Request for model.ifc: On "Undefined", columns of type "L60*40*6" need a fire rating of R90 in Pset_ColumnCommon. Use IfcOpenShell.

First a look at what the model holds.

```python
import ifcopenshell
import ifcopenshell.util.element

model = ifcopenshell.open("model.ifc")
print(model.schema)
storey = next(s for s in model.by_type("IfcBuildingStorey") if s.Name == "Undefined")
columns = [e for e in ifcopenshell.util.element.get_decomposition(storey) if e.is_a("IfcColumn")]
seen = {}
for e in columns:
    element_type = ifcopenshell.util.element.get_type(e)
    key = (element_type.Name if element_type != e and element_type else None, ifcopenshell.util.element.get_pset(e, "Pset_ColumnCommon", "FireRating"))
    seen[key] = seen.get(key, 0) + 1
for (name, value), count in sorted(seen.items(), key=str):
    print(count, "x", name, "|", value)
```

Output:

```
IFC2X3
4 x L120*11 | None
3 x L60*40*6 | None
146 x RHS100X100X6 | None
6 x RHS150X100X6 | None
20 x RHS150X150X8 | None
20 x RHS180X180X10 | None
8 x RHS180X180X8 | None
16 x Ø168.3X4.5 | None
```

```python
import ifcopenshell
import ifcopenshell.api.pset
import ifcopenshell.util.element

model = ifcopenshell.open("model.ifc")

storey = next(s for s in model.by_type("IfcBuildingStorey") if s.Name == "Undefined")
columns = [e for e in ifcopenshell.util.element.get_decomposition(storey) if e.is_a("IfcColumn")]

count = 0
for e in columns:
    element_type = ifcopenshell.util.element.get_type(e)
    if element_type in (None, e) or element_type.Name != "L60*40*6":
        continue
    # add_pset returns the element's existing set when there is one.
    pset = ifcopenshell.api.pset.add_pset(model, product=e, name="Pset_ColumnCommon")
    ifcopenshell.api.pset.edit_pset(model, pset=pset, properties={"FireRating": "R90"})
    count += 1

print(count, "columns updated")

model.write("model_rev.ifc")
```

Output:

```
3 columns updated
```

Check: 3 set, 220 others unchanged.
